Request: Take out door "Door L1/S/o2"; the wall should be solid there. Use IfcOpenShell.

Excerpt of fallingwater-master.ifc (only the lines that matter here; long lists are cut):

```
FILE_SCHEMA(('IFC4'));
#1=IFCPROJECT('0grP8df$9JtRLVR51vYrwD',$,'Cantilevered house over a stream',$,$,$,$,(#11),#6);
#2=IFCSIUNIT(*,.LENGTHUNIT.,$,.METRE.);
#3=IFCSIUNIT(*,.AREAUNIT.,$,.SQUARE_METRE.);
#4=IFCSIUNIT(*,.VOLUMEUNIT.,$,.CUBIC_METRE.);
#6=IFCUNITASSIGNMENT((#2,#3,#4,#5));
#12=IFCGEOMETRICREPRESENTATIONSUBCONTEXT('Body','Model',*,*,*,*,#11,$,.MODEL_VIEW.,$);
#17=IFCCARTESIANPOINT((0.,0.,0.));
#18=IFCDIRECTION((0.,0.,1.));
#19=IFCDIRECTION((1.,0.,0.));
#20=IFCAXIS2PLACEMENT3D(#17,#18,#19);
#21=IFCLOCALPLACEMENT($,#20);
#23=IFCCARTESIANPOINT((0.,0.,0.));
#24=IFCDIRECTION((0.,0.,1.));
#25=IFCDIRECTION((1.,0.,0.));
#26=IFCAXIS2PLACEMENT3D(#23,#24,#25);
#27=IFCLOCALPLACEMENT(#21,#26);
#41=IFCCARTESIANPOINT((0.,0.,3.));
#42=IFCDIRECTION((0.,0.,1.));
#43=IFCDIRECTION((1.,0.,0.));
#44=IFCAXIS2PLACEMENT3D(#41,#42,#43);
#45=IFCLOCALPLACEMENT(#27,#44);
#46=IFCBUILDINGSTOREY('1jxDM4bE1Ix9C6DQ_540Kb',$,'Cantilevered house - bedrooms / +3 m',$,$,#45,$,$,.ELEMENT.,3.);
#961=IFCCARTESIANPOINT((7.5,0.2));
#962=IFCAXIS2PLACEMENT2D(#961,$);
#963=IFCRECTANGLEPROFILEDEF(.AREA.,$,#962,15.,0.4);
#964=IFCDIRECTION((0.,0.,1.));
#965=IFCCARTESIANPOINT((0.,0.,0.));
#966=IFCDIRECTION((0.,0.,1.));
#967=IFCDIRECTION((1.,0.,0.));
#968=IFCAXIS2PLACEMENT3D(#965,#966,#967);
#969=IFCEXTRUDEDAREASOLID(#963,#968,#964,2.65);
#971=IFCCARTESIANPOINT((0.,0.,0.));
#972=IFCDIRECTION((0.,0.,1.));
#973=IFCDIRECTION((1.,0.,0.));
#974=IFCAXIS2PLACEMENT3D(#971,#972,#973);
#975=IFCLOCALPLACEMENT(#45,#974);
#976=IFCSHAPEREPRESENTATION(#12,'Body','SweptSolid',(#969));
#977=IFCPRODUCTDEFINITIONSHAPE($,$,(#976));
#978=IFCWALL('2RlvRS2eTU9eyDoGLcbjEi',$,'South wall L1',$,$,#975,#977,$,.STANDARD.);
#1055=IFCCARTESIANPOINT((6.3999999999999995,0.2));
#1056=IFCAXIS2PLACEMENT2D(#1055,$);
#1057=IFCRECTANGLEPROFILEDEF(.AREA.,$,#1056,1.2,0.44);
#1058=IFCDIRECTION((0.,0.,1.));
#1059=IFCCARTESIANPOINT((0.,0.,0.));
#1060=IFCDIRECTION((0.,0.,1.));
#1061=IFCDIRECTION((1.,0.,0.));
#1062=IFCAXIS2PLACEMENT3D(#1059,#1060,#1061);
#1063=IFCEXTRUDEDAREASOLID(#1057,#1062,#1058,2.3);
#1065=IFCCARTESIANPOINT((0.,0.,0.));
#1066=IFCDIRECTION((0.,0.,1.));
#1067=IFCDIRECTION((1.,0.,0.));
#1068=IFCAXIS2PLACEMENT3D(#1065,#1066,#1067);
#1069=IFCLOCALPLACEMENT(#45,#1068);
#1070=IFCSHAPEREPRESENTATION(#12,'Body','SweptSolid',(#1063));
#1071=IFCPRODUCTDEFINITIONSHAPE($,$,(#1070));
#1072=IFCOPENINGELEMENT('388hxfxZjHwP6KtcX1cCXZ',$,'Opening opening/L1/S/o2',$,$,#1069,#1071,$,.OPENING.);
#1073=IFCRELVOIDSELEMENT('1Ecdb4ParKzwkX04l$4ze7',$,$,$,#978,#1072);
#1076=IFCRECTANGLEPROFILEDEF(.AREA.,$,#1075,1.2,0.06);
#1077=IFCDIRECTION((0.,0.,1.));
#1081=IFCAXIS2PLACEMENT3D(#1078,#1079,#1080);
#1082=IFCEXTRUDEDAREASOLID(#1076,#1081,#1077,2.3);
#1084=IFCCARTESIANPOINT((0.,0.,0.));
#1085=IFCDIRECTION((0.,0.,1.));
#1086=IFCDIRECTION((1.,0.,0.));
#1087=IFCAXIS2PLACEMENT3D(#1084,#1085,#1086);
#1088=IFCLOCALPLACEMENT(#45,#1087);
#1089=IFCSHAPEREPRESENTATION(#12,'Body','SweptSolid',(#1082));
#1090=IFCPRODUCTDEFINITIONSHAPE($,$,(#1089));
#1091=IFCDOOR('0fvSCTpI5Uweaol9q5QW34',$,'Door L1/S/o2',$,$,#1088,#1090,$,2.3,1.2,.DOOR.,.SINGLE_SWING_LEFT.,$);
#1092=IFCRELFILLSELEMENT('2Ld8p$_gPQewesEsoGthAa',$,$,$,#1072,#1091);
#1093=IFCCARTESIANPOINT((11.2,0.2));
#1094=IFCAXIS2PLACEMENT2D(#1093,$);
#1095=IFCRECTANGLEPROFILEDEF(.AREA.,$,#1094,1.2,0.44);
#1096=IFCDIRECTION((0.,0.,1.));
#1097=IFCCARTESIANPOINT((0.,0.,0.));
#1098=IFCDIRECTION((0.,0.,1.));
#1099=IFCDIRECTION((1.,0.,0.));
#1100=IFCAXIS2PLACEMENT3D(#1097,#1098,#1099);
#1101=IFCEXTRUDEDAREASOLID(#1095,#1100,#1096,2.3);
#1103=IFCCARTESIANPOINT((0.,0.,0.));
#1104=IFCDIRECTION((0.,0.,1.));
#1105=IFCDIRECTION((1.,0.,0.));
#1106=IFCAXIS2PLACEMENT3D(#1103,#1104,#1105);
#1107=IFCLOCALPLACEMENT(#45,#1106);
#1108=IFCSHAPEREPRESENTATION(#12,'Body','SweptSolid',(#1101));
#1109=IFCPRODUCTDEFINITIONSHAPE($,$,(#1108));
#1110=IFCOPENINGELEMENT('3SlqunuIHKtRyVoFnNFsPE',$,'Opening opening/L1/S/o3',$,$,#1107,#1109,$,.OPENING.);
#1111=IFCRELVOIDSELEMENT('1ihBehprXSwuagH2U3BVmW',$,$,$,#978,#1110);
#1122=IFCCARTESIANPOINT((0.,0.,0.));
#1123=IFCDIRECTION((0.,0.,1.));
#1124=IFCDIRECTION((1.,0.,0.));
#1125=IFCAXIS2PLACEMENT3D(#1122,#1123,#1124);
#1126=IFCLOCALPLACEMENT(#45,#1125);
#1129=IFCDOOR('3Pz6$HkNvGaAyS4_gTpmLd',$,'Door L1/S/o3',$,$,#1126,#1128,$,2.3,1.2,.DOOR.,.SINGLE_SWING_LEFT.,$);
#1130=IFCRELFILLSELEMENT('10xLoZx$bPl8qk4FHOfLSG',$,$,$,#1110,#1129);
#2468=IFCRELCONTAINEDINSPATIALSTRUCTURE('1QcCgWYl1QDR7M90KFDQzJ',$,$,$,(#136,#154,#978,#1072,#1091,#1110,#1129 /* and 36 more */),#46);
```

```python
import ifcopenshell
import ifcopenshell.api.feature
import ifcopenshell.api.root
import ifcopenshell.geom
import ifcopenshell.util.shape

model = ifcopenshell.open("fallingwater-master.ifc")
settings = ifcopenshell.geom.settings()


def volume(element):
    """Net volume in cubic metres, openings subtracted."""
    shape = ifcopenshell.geom.create_shape(settings, element)
    return ifcopenshell.util.shape.get_volume(shape.geometry)


door = model.by_guid("0fvSCTpI5Uweaol9q5QW34")
opening = door.FillsVoids[0].RelatingOpeningElement
wall = opening.VoidsElements[0].RelatingBuildingElement
before = volume(wall)

ifcopenshell.api.root.remove_product(model, product=door)
ifcopenshell.api.feature.remove_feature(model, feature=opening)

after = volume(wall)

print(f"wall volume {before:.3f} -> {after:.3f} m3")

model.write("fallingwater-master_rev.ifc")
```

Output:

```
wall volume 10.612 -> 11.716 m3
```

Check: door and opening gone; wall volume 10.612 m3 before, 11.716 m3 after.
